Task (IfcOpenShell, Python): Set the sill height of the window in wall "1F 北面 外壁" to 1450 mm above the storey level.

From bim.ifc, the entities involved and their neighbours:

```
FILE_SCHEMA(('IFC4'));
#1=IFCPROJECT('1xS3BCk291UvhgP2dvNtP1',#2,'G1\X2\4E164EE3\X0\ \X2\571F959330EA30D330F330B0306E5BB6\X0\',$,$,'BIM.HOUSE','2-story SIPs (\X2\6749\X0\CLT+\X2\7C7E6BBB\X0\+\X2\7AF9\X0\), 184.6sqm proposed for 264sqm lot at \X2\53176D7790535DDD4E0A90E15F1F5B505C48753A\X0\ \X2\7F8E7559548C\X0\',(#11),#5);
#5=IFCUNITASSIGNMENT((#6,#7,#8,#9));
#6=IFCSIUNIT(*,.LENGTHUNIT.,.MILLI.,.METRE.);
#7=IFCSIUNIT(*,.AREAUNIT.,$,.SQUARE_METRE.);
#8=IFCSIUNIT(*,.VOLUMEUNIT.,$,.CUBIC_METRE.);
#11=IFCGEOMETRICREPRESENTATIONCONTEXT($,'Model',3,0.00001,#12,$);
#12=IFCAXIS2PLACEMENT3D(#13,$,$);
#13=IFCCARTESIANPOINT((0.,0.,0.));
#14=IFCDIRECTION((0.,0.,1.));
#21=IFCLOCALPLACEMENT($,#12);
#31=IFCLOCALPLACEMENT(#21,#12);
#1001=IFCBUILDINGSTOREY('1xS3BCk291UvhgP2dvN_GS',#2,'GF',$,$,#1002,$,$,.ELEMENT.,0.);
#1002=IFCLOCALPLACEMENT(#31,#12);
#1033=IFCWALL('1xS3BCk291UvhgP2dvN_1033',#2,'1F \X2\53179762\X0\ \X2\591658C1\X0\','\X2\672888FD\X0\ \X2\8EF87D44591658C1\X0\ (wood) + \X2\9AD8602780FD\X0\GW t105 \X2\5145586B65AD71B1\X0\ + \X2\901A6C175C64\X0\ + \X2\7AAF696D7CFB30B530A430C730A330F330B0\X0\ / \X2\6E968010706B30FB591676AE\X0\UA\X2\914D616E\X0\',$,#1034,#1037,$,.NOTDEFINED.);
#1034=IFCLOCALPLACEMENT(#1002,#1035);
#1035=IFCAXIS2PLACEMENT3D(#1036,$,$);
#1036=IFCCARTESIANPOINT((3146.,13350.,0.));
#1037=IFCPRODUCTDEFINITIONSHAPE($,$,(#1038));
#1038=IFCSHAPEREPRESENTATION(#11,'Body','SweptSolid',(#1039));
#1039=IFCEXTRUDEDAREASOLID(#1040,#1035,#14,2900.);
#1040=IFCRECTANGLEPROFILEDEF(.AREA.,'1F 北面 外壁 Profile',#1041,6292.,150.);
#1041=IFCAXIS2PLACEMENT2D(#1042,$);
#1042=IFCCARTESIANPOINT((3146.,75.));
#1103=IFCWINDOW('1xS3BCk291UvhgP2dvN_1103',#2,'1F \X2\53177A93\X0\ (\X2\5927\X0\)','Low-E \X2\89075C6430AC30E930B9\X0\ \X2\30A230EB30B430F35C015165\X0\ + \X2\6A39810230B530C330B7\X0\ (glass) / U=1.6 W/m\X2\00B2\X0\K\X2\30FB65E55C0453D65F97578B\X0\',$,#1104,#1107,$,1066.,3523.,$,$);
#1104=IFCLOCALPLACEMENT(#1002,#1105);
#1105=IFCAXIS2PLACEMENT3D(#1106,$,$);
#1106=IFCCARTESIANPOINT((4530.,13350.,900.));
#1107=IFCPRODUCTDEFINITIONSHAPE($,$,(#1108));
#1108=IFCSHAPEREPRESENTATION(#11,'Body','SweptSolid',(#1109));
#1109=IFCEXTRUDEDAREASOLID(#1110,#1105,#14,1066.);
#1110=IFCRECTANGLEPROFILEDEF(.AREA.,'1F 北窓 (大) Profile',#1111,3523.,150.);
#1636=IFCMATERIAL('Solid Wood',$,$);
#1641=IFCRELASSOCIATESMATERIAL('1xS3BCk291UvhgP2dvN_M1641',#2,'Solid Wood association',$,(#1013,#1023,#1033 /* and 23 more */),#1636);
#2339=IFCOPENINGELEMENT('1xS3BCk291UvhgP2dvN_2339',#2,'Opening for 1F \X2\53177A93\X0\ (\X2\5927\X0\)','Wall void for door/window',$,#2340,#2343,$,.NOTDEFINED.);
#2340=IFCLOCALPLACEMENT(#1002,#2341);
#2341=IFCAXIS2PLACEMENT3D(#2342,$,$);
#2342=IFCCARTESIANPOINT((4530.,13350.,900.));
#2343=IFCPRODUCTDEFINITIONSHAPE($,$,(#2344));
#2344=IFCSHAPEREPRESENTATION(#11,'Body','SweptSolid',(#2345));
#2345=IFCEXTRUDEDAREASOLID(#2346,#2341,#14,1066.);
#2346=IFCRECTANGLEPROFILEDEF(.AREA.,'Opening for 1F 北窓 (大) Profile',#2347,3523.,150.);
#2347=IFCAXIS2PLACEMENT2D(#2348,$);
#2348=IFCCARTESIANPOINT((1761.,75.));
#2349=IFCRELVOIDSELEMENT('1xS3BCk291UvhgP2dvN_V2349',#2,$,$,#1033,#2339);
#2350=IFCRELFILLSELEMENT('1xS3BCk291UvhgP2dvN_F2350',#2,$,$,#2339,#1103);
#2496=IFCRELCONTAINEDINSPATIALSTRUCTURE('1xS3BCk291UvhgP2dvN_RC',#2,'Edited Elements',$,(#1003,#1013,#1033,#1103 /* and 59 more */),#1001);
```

```python
import numpy as np
import ifcopenshell
import ifcopenshell.api.geometry
import ifcopenshell.geom
import ifcopenshell.util.element
import ifcopenshell.util.placement
import ifcopenshell.util.shape
import ifcopenshell.util.unit

model = ifcopenshell.open("bim.ifc")
unit_scale = ifcopenshell.util.unit.calculate_unit_scale(model)

window = model.by_guid("1xS3BCk291UvhgP2dvN_1103")
opening = window.FillsVoids[0].RelatingOpeningElement
storey = ifcopenshell.util.element.get_container(window, ifc_class="IfcBuildingStorey")
level = ifcopenshell.util.placement.get_local_placement(storey.ObjectPlacement)[2, 3]

# The opening's origin need not be at the sill, so measure its lowest point.
shape = ifcopenshell.geom.create_shape(ifcopenshell.geom.settings(), opening)
bottom = ifcopenshell.util.shape.get_shape_bottom_elevation(shape, shape.geometry) / unit_scale
dz = level + 1450.0 - bottom

shift = np.array([0.0, 0.0, dz])
# The window is not placed relative to its opening, so move both.
for product in (opening, window):
    matrix = ifcopenshell.util.placement.get_local_placement(product.ObjectPlacement)
    matrix[:3, 3] += shift
    ifcopenshell.api.geometry.edit_object_placement(model, product=product, matrix=matrix, is_si=False)

print(f"moved by {dz * unit_scale:+.3f} m")

model.write("bim_rev.ifc")
```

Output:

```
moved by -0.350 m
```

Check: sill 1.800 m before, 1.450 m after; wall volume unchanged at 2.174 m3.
